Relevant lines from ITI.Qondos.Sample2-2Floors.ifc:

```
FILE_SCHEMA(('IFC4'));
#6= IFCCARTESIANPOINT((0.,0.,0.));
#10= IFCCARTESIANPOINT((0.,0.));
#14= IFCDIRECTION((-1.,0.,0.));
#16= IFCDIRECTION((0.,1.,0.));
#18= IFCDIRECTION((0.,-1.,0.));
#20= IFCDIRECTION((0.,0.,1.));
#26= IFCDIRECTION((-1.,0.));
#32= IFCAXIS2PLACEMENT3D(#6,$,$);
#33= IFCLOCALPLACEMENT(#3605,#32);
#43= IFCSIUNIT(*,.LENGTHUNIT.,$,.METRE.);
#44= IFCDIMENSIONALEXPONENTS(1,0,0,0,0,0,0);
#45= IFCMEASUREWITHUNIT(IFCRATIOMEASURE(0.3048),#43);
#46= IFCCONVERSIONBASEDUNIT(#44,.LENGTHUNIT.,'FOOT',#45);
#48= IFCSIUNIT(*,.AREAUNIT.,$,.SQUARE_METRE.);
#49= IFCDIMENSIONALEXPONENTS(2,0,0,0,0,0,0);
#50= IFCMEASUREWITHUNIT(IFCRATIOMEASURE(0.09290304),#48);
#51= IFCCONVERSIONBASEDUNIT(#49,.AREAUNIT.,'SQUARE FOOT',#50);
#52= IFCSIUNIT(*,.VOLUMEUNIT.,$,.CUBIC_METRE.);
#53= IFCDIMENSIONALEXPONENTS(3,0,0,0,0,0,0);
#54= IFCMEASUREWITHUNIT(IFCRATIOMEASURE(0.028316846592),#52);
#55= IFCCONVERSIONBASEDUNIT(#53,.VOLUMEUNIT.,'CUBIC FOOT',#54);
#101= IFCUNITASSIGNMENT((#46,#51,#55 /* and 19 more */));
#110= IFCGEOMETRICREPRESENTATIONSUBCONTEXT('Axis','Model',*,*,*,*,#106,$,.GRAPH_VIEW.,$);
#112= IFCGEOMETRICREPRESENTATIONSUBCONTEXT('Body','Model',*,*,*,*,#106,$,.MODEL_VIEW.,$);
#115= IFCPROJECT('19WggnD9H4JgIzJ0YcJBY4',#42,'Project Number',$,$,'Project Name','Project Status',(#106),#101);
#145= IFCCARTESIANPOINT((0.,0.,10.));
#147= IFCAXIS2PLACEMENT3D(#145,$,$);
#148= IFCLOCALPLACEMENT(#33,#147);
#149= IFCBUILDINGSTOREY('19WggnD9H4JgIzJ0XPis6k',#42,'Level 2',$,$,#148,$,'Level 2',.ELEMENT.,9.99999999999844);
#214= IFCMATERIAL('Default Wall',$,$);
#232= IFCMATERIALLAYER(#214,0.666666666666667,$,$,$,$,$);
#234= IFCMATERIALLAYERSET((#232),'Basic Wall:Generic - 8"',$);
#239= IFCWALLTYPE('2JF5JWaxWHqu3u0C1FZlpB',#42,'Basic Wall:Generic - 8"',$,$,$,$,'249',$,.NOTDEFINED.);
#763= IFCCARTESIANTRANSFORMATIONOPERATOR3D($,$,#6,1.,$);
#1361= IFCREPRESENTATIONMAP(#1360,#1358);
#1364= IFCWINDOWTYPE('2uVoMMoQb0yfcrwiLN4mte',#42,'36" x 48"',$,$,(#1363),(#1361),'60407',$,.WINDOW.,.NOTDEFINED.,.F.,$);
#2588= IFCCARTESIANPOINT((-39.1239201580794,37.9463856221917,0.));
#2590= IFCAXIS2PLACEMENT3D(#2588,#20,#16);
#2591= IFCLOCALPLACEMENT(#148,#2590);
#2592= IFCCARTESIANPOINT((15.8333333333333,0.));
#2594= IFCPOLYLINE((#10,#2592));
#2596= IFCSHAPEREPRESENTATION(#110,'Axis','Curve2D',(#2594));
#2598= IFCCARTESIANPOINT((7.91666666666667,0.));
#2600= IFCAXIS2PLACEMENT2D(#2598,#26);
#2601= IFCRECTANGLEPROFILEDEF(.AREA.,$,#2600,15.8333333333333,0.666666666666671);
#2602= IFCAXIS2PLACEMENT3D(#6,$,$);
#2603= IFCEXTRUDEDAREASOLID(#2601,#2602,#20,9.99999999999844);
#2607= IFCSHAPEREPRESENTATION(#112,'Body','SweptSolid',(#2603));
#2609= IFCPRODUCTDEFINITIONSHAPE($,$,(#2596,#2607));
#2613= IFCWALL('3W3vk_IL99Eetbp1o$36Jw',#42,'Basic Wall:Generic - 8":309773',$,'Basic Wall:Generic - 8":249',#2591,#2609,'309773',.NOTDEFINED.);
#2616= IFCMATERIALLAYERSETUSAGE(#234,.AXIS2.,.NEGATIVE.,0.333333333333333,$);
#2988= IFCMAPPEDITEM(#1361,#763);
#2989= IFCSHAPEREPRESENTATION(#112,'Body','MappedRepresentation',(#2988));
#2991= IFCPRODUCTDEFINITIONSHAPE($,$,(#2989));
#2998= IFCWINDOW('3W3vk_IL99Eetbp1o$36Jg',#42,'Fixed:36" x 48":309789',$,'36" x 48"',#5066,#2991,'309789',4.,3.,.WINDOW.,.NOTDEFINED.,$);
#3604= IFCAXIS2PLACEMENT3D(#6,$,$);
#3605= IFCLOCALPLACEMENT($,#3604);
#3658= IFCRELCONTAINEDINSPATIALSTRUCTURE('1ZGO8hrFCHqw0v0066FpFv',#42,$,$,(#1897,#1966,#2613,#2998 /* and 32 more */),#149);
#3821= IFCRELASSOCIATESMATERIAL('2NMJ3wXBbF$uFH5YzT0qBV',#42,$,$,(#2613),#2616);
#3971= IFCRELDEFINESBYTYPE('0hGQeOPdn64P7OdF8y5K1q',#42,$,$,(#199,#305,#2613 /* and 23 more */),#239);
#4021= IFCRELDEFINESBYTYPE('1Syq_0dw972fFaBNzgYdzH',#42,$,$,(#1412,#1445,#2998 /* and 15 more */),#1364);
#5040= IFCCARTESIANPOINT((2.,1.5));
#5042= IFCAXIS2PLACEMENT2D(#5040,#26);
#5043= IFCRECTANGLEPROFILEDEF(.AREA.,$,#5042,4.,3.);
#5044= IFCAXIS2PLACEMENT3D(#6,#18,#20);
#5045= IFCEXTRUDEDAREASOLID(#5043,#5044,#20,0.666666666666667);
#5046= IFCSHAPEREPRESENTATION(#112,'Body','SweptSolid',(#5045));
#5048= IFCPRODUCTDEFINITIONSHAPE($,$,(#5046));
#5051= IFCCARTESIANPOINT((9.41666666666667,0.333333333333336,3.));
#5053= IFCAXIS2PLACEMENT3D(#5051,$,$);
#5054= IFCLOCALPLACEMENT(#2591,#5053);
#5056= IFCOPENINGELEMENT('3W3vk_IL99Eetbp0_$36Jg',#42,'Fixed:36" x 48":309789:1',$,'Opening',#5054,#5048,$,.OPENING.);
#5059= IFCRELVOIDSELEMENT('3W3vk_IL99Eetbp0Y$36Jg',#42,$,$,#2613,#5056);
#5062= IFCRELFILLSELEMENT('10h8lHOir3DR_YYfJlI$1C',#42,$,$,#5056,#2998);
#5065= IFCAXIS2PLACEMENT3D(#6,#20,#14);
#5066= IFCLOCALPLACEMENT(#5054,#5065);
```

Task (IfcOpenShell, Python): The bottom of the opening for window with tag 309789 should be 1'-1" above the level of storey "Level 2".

```python
import numpy as np
import ifcopenshell
import ifcopenshell.api.geometry
import ifcopenshell.geom
import ifcopenshell.util.element
import ifcopenshell.util.placement
import ifcopenshell.util.shape
import ifcopenshell.util.unit

model = ifcopenshell.open("ITI.Qondos.Sample2-2Floors.ifc")
unit_scale = ifcopenshell.util.unit.calculate_unit_scale(model)

window = model.by_guid("3W3vk_IL99Eetbp1o$36Jg")
opening = window.FillsVoids[0].RelatingOpeningElement
storey = ifcopenshell.util.element.get_container(window, ifc_class="IfcBuildingStorey")
level = ifcopenshell.util.placement.get_local_placement(storey.ObjectPlacement)[2, 3]

# The opening's origin need not be at the sill, so measure its lowest point.
shape = ifcopenshell.geom.create_shape(ifcopenshell.geom.settings(), opening)
bottom = ifcopenshell.util.shape.get_shape_bottom_elevation(shape, shape.geometry) / unit_scale
dz = level + 13 * 0.0254 / unit_scale - bottom

shift = np.array([0.0, 0.0, dz])
# The window is placed relative to its opening, so it follows when the opening moves.
matrix = ifcopenshell.util.placement.get_local_placement(opening.ObjectPlacement)
matrix[:3, 3] += shift
ifcopenshell.api.geometry.edit_object_placement(
    model, product=opening, matrix=matrix, is_si=False, should_transform_children=True
)

print(f"moved by {dz * unit_scale:+.3f} m")

model.write("ITI.Qondos.Sample2-2Floors_updated.ifc")
```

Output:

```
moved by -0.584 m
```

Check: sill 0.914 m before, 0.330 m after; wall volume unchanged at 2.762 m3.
